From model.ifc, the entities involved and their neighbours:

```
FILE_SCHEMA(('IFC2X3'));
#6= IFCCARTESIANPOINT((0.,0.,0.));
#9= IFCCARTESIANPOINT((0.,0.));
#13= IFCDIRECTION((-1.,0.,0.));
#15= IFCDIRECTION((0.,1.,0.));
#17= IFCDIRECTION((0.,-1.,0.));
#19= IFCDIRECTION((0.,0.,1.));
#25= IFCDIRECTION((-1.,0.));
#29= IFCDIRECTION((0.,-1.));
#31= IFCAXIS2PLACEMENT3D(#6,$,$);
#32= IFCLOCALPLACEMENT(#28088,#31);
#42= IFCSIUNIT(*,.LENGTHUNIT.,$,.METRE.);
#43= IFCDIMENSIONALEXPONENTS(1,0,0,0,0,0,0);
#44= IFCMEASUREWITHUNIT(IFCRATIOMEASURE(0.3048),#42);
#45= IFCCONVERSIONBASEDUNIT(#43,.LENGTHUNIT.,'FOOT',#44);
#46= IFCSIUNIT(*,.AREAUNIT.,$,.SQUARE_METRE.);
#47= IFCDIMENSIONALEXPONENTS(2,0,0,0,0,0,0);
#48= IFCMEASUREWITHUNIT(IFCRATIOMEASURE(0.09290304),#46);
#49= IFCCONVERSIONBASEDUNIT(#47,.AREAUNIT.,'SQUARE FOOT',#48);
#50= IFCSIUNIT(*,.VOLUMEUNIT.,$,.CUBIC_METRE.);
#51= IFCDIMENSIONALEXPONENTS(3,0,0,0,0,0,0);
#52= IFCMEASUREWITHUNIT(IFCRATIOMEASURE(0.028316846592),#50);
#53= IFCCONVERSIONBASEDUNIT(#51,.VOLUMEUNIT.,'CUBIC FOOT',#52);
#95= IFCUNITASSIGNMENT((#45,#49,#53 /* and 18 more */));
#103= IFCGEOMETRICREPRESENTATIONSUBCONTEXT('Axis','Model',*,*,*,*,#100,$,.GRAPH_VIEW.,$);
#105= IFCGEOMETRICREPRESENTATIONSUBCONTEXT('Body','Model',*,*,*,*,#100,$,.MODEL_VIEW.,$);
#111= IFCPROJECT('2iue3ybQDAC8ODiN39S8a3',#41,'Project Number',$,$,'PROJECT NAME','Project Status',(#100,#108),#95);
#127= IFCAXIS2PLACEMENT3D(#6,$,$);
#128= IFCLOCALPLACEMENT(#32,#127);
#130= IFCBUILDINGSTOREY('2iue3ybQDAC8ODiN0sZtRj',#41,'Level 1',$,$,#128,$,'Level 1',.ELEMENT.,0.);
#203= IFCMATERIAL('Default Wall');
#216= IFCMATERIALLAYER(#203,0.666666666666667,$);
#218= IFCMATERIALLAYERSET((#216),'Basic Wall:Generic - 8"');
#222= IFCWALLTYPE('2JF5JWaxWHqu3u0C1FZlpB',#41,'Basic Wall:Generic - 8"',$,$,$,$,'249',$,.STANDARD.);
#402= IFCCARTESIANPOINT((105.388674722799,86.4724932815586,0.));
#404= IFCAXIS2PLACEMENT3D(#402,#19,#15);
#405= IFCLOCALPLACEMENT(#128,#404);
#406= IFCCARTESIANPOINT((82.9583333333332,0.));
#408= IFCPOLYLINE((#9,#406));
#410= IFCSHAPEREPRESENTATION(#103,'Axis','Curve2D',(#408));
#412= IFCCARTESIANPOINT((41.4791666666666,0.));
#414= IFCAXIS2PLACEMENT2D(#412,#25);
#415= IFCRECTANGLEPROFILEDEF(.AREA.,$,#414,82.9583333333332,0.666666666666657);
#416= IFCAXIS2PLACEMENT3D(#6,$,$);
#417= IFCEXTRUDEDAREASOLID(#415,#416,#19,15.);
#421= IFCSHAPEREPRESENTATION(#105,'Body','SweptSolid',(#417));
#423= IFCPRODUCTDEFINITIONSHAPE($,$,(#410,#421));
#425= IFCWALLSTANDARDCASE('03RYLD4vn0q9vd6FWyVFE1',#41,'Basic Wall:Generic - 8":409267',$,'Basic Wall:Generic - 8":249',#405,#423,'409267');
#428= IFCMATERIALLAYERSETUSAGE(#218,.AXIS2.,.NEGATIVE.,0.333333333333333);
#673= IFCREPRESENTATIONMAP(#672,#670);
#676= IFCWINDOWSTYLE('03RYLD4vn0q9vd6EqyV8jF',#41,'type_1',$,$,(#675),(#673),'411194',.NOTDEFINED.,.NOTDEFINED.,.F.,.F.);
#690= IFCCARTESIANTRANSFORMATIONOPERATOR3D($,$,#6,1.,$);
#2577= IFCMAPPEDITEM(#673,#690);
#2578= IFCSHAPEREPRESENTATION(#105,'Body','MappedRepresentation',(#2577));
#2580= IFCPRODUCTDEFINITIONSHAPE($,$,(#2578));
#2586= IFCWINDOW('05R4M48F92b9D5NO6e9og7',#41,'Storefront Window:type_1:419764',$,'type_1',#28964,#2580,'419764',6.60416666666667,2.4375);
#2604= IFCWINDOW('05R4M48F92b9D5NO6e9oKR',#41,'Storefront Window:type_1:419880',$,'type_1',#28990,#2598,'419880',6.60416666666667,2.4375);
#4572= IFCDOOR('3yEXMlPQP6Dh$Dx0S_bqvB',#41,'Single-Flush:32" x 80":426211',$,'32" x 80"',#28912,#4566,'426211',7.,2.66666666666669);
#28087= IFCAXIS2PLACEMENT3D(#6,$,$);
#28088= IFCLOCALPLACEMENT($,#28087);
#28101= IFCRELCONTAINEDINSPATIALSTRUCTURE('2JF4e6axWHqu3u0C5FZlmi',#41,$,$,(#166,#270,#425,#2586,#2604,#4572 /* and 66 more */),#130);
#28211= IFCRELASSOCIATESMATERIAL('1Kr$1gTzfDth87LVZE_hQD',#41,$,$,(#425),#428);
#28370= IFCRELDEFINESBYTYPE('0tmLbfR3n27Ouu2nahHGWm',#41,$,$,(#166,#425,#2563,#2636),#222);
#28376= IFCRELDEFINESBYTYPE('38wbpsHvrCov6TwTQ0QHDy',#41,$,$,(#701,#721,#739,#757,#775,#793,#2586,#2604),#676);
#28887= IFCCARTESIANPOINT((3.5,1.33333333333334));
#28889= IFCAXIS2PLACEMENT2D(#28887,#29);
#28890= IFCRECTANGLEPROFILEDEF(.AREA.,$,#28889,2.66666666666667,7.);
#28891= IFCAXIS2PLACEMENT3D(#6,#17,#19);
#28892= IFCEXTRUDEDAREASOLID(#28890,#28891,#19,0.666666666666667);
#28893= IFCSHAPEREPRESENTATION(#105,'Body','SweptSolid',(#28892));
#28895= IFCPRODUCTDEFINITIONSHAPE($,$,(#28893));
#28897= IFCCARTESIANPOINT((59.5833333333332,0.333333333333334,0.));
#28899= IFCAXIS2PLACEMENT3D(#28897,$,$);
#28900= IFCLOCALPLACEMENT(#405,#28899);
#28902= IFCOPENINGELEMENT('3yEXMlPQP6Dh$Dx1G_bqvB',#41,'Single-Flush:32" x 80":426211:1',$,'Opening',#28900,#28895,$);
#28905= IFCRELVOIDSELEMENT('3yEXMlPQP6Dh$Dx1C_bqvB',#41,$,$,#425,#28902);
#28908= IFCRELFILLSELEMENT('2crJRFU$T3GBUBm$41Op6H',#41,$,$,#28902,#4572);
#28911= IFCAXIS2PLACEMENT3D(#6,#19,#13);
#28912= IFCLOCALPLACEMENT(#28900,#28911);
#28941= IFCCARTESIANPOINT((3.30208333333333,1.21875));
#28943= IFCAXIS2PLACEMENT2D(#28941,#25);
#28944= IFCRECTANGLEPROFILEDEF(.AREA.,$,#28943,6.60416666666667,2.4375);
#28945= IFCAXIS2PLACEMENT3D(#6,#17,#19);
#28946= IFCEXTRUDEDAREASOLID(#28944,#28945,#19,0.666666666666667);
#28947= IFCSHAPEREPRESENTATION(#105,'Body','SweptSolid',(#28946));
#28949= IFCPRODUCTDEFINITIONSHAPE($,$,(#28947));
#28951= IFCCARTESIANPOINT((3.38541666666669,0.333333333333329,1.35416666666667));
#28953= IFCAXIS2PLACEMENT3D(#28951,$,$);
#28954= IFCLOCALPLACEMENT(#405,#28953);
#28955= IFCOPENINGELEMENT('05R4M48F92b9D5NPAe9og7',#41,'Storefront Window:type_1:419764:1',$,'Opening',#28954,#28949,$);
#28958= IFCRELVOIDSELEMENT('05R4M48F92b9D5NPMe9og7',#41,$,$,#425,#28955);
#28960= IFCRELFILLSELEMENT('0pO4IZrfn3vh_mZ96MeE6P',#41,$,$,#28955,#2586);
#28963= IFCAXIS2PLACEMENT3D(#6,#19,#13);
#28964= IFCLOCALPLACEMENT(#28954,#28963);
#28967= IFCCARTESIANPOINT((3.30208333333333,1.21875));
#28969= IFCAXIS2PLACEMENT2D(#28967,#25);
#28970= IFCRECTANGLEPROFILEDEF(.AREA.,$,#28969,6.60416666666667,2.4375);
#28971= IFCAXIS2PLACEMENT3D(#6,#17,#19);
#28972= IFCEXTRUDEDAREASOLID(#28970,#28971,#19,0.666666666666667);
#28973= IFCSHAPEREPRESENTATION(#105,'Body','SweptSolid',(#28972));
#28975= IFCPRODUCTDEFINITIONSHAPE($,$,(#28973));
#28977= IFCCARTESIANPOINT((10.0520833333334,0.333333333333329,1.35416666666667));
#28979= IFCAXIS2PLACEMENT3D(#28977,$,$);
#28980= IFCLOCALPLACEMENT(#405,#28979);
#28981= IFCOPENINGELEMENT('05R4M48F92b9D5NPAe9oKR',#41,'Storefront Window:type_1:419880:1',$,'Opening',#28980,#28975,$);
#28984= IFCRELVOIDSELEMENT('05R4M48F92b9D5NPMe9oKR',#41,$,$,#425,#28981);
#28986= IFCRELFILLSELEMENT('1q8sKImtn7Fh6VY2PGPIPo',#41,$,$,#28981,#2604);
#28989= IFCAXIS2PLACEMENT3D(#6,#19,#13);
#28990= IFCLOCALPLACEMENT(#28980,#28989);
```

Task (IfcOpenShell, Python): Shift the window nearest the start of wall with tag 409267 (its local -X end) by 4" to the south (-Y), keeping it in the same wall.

```python
import ifcopenshell
import ifcopenshell.api.geometry
import ifcopenshell.util.placement
import ifcopenshell.util.unit

model = ifcopenshell.open("model.ifc")
unit_scale = ifcopenshell.util.unit.calculate_unit_scale(model)

window = model.by_guid("05R4M48F92b9D5NO6e9og7")
opening = window.FillsVoids[0].RelatingOpeningElement
wall = opening.VoidsElements[0].RelatingBuildingElement

wall_matrix = ifcopenshell.util.placement.get_local_placement(wall.ObjectPlacement)
shift = wall_matrix[:3, 0] * -4 * 0.0254 / unit_scale
before = ifcopenshell.util.placement.get_local_placement(window.ObjectPlacement)[:3, 3].copy()

# The window is placed relative to its opening, so it follows when the opening moves.
matrix = ifcopenshell.util.placement.get_local_placement(opening.ObjectPlacement)
matrix[:3, 3] += shift
ifcopenshell.api.geometry.edit_object_placement(
    model, product=opening, matrix=matrix, is_si=False, should_transform_children=True
)

after = ifcopenshell.util.placement.get_local_placement(window.ObjectPlacement)[:3, 3]
print("window moved by", (after - before).round(3) + 0.0)

model.write("model_updated.ifc")
```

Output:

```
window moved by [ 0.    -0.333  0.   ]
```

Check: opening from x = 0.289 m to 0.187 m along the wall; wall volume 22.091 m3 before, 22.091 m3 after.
